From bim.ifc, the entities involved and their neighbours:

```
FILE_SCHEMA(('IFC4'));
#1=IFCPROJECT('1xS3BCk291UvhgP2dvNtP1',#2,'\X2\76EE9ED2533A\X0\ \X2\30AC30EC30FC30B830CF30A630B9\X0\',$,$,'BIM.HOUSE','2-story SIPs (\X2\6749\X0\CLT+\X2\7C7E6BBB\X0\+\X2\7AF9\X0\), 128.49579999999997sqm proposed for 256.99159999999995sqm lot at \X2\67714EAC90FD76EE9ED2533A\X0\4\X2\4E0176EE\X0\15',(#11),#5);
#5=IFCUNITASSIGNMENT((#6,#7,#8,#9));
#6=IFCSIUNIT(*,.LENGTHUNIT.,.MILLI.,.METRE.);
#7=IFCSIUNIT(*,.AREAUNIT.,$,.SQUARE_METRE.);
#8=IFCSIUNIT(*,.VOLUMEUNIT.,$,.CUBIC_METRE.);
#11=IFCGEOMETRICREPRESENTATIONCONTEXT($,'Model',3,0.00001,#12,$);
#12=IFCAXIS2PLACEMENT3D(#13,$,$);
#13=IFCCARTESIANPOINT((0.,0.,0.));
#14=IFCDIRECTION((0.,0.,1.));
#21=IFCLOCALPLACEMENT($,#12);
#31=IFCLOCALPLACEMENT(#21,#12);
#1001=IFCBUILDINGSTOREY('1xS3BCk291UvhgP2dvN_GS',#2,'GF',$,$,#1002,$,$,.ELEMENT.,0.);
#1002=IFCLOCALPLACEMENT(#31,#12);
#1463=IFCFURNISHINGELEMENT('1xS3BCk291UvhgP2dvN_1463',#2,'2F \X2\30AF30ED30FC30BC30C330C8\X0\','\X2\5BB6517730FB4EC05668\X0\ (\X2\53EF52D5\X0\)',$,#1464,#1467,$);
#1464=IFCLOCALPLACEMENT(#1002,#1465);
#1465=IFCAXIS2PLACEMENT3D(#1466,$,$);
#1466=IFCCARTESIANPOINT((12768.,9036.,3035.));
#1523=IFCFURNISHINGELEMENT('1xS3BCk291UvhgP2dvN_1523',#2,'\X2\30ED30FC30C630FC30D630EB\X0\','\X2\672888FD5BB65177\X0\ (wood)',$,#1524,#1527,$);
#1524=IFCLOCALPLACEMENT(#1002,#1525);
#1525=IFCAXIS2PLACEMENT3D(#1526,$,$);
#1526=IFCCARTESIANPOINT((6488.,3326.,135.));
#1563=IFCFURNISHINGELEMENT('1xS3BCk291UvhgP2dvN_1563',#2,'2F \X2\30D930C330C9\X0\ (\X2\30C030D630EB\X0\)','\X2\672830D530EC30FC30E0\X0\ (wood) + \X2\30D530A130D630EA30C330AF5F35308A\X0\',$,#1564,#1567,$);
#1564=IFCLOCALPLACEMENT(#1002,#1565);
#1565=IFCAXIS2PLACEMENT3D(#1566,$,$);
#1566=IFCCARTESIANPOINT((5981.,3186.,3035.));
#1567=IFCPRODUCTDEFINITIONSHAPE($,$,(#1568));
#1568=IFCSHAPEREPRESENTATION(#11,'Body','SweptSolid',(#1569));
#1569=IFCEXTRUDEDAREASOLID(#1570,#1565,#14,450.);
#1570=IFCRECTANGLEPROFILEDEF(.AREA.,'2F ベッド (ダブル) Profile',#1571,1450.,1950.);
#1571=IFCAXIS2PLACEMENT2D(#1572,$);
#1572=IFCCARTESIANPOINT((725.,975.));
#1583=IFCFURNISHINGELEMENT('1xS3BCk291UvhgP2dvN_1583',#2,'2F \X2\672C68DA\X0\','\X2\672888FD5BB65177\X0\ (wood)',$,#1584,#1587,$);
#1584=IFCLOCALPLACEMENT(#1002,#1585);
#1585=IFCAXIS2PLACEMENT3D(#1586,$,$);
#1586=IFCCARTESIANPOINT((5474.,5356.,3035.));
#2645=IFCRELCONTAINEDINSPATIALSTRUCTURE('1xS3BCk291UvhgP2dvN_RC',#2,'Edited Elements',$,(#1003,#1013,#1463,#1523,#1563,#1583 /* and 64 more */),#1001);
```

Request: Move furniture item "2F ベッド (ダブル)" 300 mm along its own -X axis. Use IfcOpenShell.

```python
import ifcopenshell
import ifcopenshell.api.geometry
import ifcopenshell.util.placement

model = ifcopenshell.open("bim.ifc")

item = model.by_id(1563)
matrix = ifcopenshell.util.placement.get_local_placement(item.ObjectPlacement)
matrix[:3, 3] -= matrix[:3, 0] * 300.0
ifcopenshell.api.geometry.edit_object_placement(model, product=item, matrix=matrix, is_si=False)

print(ifcopenshell.util.placement.get_local_placement(item.ObjectPlacement).round(3) + 0.0)

model.write("bim_rev.ifc")
```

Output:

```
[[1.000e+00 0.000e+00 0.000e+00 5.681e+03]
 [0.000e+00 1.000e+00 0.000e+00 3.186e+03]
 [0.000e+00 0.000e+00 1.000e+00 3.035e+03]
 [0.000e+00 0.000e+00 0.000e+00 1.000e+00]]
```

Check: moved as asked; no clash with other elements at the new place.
